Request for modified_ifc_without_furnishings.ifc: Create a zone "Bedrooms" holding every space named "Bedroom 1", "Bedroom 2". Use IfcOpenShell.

First a look at what the model holds.

```python
import ifcopenshell

model = ifcopenshell.open("modified_ifc_without_furnishings.ifc")
print(model.schema)
seen = {}
for space in model.by_type("IfcSpace"):
    seen[space.LongName] = seen.get(space.LongName, 0) + 1
for name, count in sorted(seen.items(), key=str):
    print(count, "x", name)
print("zones:", [z.Name for z in model.by_type("IfcZone")][:20])
```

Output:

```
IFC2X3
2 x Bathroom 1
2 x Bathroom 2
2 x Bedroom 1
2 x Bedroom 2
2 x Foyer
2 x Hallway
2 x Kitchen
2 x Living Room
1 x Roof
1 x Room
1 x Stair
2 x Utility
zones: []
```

```python
import ifcopenshell
import ifcopenshell.api.group
import ifcopenshell.api.root

model = ifcopenshell.open("modified_ifc_without_furnishings.ifc")

names = {"Bedroom 1", "Bedroom 2"}
spaces = [s for s in model.by_type("IfcSpace") if s.LongName in names]

zone = ifcopenshell.api.root.create_entity(model, ifc_class="IfcZone", name="Bedrooms")
ifcopenshell.api.group.assign_group(model, products=spaces, group=zone)
print(len(spaces), "spaces in", zone.Name)

model.write("modified_ifc_without_furnishings_updated.ifc")
```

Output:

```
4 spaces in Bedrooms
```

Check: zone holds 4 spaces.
